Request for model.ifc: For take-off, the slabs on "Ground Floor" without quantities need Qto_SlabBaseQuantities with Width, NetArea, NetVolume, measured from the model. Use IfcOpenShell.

First a look at what the model holds.

```python
import ifcopenshell
import ifcopenshell.util.element
import ifcopenshell.util.unit

model = ifcopenshell.open("model.ifc")
print(model.schema)
for unit_type in ("LENGTHUNIT", "AREAUNIT", "VOLUMEUNIT"):
    print(unit_type, ifcopenshell.util.unit.calculate_unit_scale(model, unit_type))
storey = next(s for s in model.by_type("IfcBuildingStorey") if s.Name == "Ground Floor")
slabs = [e for e in ifcopenshell.util.element.get_decomposition(storey) if e.is_a("IfcSlab")]
for e in sorted(slabs, key=lambda e: e.id()):
    print(e.id(), e.is_a(), e.Name, list(ifcopenshell.util.element.get_psets(e, qtos_only=True)), sep=" | ")
```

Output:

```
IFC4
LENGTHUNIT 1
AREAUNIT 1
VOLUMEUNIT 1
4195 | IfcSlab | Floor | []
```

```python
import ifcopenshell
import ifcopenshell.api.pset
import ifcopenshell.geom
import ifcopenshell.util.element
import ifcopenshell.util.shape
import ifcopenshell.util.unit

model = ifcopenshell.open("model.ifc")
unit_scale = ifcopenshell.util.unit.calculate_unit_scale(model)
area_scale = ifcopenshell.util.unit.calculate_unit_scale(model, "AREAUNIT")
volume_scale = ifcopenshell.util.unit.calculate_unit_scale(model, "VOLUMEUNIT")
settings = ifcopenshell.geom.settings()

storey = next(s for s in model.by_type("IfcBuildingStorey") if s.Name == "Ground Floor")
slabs = [e for e in ifcopenshell.util.element.get_decomposition(storey) if e.is_a("IfcSlab")]

for e in sorted(slabs, key=lambda e: e.id()):
    if ifcopenshell.util.element.get_psets(e, qtos_only=True, should_inherit=False):
        continue
    # Geometry comes back in metres, in the element's own axes.
    shape = ifcopenshell.geom.create_shape(settings, e)
    values = {
        "Width": ifcopenshell.util.shape.get_z(shape.geometry) / unit_scale,
        "NetArea": ifcopenshell.util.shape.get_footprint_area(shape.geometry) / area_scale,
        "NetVolume": ifcopenshell.util.shape.get_volume(shape.geometry) / volume_scale,
    }
    qto = ifcopenshell.api.pset.add_qto(model, product=e, name="Qto_SlabBaseQuantities")
    ifcopenshell.api.pset.edit_qto(model, qto=qto, properties=values)
    print(e.id(), {k: round(v, 3) for k, v in values.items()})

model.write("model-out.ifc")
```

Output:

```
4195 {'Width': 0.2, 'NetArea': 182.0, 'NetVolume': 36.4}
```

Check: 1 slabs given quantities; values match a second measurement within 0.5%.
